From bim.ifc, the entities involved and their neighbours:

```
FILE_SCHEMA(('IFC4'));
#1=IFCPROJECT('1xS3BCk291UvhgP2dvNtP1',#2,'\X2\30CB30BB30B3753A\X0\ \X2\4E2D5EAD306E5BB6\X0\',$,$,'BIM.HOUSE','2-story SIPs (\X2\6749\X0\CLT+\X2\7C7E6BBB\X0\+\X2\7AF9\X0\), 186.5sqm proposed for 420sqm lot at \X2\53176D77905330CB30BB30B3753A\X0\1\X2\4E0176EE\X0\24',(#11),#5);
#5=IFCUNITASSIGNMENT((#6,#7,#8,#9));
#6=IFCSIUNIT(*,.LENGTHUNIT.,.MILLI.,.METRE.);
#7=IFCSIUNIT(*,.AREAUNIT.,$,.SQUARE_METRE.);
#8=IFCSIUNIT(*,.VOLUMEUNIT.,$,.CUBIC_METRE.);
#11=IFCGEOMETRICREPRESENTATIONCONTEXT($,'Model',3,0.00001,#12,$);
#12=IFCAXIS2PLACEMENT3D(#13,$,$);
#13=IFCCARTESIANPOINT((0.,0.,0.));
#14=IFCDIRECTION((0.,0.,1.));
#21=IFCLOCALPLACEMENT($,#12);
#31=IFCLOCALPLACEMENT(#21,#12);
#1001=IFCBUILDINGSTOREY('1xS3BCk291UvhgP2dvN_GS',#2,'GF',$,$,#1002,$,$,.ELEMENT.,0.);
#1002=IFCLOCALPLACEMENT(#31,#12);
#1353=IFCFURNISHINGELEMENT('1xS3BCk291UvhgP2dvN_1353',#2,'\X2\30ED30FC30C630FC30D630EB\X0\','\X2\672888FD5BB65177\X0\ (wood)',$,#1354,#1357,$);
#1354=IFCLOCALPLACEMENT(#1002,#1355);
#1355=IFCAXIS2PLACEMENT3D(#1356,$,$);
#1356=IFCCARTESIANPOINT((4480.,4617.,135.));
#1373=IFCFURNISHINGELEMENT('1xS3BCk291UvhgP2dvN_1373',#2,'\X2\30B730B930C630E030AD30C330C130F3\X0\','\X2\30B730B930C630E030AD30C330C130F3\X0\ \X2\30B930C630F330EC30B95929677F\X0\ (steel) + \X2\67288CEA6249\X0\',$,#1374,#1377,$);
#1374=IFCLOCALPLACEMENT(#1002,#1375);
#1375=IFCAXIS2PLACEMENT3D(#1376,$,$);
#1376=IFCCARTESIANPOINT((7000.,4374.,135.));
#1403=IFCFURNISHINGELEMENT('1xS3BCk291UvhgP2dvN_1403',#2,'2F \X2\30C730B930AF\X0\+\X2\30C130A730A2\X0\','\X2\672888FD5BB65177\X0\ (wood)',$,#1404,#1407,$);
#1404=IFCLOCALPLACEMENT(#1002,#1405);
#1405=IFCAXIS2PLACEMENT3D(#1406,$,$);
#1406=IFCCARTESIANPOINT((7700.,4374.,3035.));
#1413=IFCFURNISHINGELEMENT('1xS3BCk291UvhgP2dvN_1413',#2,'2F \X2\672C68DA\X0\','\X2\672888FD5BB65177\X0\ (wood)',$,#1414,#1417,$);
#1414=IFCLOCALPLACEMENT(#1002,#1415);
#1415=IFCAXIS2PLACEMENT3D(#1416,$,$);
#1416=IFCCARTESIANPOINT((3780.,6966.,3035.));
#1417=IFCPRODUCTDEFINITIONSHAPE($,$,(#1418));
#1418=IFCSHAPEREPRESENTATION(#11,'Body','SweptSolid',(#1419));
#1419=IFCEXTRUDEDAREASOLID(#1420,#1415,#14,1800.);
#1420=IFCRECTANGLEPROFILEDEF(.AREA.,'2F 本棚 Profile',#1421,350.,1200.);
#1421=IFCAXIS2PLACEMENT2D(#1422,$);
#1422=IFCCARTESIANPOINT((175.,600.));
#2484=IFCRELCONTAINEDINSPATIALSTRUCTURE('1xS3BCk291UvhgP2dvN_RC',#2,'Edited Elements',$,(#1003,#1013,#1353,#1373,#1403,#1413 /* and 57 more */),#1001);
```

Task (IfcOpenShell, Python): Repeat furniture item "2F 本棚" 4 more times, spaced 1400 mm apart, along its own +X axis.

```python
import ifcopenshell
import ifcopenshell.api.geometry
import ifcopenshell.api.root
import ifcopenshell.util.element
import ifcopenshell.util.placement

model = ifcopenshell.open("bim.ifc")


def reuse_history(source, copy):
    """copy_class also copies each property set's owner history, people and application; keep the originals."""
    for rel in copy.IsDefinedBy:
        if rel.is_a("IfcRelDefinesByProperties") and (history := rel.RelatingPropertyDefinition.OwnerHistory):
            rel.RelatingPropertyDefinition.OwnerHistory = source.OwnerHistory
            ifcopenshell.util.element.remove_deep2(model, history)


source = model.by_guid("1xS3BCk291UvhgP2dvN_1413")
base = ifcopenshell.util.placement.get_local_placement(source.ObjectPlacement)
step = base[:3, 0] * 1400.0

for i in range(1, 5):
    copy = ifcopenshell.api.root.copy_class(model, product=source)
    copy.Representation = ifcopenshell.util.element.copy_deep(
        model, source.Representation, exclude=["IfcGeometricRepresentationContext", "IfcRepresentationMap"]
    )
    reuse_history(source, copy)
    matrix = base.copy()
    matrix[:3, 3] += i * step
    print("added at", matrix[:3, 3].round(3) + 0.0)
    ifcopenshell.api.geometry.edit_object_placement(model, product=copy, matrix=matrix, is_si=False)

model.write("bim_updated.ifc")
```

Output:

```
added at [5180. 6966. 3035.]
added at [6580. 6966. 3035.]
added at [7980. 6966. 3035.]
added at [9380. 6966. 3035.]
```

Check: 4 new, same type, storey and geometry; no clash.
